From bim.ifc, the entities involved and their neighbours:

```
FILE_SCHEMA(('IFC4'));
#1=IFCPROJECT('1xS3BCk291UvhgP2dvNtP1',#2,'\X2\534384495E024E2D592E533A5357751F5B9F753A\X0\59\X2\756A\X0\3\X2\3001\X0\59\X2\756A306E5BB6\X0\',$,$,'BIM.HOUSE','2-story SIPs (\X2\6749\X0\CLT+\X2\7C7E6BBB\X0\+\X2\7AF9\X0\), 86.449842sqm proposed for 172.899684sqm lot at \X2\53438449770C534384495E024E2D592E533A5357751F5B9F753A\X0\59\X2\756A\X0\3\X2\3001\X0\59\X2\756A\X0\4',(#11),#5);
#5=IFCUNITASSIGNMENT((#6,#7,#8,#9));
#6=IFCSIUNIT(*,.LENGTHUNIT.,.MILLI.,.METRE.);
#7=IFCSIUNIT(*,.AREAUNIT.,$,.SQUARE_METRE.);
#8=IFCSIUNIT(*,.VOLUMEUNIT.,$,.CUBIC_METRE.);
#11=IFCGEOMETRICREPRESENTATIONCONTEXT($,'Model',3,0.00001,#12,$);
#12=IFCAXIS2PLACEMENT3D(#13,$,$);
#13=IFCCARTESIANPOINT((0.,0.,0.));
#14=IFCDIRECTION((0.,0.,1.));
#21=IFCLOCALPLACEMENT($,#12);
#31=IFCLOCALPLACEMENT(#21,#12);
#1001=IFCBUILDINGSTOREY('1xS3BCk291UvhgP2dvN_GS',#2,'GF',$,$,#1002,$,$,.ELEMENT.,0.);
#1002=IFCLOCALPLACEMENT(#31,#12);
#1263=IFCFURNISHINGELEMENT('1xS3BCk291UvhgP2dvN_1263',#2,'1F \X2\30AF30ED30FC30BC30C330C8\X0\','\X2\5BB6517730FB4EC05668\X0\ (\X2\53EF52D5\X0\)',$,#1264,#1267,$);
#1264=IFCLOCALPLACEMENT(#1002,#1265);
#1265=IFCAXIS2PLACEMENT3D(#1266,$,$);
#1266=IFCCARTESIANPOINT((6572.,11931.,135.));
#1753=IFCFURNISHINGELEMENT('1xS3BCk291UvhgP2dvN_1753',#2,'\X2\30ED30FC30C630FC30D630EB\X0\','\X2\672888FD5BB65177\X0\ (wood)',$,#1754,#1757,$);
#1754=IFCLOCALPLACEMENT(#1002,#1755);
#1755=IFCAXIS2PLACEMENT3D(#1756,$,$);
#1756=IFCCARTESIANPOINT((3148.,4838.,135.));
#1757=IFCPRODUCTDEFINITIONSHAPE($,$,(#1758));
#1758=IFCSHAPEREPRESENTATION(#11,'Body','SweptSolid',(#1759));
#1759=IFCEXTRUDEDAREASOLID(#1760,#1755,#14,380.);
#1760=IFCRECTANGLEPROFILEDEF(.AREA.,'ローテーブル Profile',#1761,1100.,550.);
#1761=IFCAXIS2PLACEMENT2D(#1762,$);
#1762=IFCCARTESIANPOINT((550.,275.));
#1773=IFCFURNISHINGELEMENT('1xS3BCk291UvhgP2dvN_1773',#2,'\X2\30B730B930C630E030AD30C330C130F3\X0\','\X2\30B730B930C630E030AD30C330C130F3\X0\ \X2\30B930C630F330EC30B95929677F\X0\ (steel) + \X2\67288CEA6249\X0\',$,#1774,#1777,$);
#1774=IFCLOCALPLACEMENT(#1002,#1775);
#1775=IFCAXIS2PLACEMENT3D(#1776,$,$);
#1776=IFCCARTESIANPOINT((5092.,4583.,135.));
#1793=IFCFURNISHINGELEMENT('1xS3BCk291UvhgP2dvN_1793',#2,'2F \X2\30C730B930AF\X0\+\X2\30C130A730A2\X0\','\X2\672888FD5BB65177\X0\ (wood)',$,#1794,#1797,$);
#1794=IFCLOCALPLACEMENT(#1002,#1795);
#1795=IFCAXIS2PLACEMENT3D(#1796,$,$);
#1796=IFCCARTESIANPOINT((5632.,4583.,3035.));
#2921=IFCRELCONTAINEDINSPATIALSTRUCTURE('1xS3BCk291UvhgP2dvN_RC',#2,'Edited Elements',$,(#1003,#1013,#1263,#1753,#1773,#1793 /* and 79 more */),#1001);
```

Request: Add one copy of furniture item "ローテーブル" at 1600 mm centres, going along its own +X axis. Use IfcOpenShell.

```python
import ifcopenshell
import ifcopenshell.api.geometry
import ifcopenshell.api.root
import ifcopenshell.util.element
import ifcopenshell.util.placement

model = ifcopenshell.open("bim.ifc")


def reuse_history(source, copy):
    """copy_class also copies each property set's owner history, people and application; keep the originals."""
    for rel in copy.IsDefinedBy:
        if rel.is_a("IfcRelDefinesByProperties") and (history := rel.RelatingPropertyDefinition.OwnerHistory):
            rel.RelatingPropertyDefinition.OwnerHistory = source.OwnerHistory
            ifcopenshell.util.element.remove_deep2(model, history)


source = model.by_guid("1xS3BCk291UvhgP2dvN_1753")
base = ifcopenshell.util.placement.get_local_placement(source.ObjectPlacement)
step = base[:3, 0] * 1600.0

for i in range(1, 2):
    copy = ifcopenshell.api.root.copy_class(model, product=source)
    copy.Representation = ifcopenshell.util.element.copy_deep(
        model, source.Representation, exclude=["IfcGeometricRepresentationContext", "IfcRepresentationMap"]
    )
    reuse_history(source, copy)
    matrix = base.copy()
    matrix[:3, 3] += i * step
    print("added at", matrix[:3, 3].round(3) + 0.0)
    ifcopenshell.api.geometry.edit_object_placement(model, product=copy, matrix=matrix, is_si=False)

model.write("bim_updated.ifc")
```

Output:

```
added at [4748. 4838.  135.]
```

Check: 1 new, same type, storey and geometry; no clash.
